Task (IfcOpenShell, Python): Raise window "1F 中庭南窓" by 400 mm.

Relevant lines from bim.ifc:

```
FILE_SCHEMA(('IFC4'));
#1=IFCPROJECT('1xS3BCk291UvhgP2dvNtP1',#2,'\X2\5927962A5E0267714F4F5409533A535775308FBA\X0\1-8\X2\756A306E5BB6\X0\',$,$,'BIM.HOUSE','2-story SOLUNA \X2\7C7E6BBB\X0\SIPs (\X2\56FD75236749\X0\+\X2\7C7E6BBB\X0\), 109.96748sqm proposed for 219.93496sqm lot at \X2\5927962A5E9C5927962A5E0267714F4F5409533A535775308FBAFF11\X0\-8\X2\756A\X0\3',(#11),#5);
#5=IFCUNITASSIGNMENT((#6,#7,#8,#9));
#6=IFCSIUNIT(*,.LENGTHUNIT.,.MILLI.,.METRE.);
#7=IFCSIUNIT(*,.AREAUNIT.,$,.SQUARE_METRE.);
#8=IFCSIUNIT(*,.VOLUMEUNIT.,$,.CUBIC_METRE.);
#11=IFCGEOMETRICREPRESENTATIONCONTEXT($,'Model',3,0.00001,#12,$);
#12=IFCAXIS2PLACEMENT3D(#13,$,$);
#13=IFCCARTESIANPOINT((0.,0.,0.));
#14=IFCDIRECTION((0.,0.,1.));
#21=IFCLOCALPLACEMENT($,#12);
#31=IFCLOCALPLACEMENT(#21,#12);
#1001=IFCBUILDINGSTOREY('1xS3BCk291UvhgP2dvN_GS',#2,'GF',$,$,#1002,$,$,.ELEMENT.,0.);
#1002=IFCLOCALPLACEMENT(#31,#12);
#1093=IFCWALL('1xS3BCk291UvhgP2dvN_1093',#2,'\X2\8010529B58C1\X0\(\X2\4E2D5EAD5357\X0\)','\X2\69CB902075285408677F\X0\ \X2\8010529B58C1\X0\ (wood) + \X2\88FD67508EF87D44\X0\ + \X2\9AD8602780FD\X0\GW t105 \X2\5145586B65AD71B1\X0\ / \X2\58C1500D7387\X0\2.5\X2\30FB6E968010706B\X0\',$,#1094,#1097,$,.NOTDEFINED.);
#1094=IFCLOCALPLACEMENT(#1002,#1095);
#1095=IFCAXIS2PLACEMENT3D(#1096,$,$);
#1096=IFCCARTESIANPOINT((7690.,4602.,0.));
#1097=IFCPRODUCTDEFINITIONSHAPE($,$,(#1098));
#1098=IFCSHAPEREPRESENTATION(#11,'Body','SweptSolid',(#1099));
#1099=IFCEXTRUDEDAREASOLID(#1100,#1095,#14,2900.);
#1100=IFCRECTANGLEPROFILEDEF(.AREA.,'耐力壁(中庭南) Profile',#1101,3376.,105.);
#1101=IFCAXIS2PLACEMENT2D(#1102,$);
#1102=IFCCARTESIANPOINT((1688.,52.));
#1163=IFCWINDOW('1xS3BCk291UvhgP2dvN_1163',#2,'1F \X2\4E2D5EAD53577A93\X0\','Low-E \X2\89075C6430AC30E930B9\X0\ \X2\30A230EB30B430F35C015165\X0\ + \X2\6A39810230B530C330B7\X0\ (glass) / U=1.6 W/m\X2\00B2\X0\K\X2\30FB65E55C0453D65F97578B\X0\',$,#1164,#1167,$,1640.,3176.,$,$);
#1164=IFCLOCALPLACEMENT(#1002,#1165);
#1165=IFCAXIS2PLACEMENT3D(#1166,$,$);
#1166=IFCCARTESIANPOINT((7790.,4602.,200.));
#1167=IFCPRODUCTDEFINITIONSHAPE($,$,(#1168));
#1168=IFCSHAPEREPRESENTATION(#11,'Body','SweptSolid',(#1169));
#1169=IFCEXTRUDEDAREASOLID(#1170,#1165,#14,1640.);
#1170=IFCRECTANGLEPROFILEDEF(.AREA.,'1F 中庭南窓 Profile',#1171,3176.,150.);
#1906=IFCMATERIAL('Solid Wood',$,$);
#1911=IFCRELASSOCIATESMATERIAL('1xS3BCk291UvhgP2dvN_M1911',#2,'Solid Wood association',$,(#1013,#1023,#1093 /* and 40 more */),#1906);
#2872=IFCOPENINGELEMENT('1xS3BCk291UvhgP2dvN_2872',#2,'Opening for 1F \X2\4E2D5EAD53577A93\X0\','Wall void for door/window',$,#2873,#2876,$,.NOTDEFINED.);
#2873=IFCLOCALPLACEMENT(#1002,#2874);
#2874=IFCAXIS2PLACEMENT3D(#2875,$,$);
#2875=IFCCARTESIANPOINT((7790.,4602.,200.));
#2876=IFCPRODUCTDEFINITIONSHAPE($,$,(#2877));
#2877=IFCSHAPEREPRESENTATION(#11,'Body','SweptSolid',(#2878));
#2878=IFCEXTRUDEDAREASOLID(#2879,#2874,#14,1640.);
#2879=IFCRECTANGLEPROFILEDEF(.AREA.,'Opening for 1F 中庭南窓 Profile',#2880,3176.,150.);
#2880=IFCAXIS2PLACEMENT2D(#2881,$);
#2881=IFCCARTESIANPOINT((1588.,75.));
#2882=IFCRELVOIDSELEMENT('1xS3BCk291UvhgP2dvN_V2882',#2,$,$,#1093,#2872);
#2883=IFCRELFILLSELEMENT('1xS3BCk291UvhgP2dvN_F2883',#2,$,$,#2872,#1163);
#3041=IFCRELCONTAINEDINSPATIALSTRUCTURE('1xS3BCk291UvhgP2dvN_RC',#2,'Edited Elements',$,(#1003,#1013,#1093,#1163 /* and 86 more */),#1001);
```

```python
import numpy as np
import ifcopenshell
import ifcopenshell.api.geometry
import ifcopenshell.util.placement
import ifcopenshell.util.unit

model = ifcopenshell.open("bim.ifc")
unit_scale = ifcopenshell.util.unit.calculate_unit_scale(model)

window = model.by_guid("1xS3BCk291UvhgP2dvN_1163")
opening = window.FillsVoids[0].RelatingOpeningElement
dz = 0.4 / unit_scale

shift = np.array([0.0, 0.0, dz])
# The window is not placed relative to its opening, so move both.
for product in (opening, window):
    matrix = ifcopenshell.util.placement.get_local_placement(product.ObjectPlacement)
    matrix[:3, 3] += shift
    ifcopenshell.api.geometry.edit_object_placement(model, product=product, matrix=matrix, is_si=False)

print(f"moved by {dz * unit_scale:+.3f} m")

model.write("bim_rev.ifc")
```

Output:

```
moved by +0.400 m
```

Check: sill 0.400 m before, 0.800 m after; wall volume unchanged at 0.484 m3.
